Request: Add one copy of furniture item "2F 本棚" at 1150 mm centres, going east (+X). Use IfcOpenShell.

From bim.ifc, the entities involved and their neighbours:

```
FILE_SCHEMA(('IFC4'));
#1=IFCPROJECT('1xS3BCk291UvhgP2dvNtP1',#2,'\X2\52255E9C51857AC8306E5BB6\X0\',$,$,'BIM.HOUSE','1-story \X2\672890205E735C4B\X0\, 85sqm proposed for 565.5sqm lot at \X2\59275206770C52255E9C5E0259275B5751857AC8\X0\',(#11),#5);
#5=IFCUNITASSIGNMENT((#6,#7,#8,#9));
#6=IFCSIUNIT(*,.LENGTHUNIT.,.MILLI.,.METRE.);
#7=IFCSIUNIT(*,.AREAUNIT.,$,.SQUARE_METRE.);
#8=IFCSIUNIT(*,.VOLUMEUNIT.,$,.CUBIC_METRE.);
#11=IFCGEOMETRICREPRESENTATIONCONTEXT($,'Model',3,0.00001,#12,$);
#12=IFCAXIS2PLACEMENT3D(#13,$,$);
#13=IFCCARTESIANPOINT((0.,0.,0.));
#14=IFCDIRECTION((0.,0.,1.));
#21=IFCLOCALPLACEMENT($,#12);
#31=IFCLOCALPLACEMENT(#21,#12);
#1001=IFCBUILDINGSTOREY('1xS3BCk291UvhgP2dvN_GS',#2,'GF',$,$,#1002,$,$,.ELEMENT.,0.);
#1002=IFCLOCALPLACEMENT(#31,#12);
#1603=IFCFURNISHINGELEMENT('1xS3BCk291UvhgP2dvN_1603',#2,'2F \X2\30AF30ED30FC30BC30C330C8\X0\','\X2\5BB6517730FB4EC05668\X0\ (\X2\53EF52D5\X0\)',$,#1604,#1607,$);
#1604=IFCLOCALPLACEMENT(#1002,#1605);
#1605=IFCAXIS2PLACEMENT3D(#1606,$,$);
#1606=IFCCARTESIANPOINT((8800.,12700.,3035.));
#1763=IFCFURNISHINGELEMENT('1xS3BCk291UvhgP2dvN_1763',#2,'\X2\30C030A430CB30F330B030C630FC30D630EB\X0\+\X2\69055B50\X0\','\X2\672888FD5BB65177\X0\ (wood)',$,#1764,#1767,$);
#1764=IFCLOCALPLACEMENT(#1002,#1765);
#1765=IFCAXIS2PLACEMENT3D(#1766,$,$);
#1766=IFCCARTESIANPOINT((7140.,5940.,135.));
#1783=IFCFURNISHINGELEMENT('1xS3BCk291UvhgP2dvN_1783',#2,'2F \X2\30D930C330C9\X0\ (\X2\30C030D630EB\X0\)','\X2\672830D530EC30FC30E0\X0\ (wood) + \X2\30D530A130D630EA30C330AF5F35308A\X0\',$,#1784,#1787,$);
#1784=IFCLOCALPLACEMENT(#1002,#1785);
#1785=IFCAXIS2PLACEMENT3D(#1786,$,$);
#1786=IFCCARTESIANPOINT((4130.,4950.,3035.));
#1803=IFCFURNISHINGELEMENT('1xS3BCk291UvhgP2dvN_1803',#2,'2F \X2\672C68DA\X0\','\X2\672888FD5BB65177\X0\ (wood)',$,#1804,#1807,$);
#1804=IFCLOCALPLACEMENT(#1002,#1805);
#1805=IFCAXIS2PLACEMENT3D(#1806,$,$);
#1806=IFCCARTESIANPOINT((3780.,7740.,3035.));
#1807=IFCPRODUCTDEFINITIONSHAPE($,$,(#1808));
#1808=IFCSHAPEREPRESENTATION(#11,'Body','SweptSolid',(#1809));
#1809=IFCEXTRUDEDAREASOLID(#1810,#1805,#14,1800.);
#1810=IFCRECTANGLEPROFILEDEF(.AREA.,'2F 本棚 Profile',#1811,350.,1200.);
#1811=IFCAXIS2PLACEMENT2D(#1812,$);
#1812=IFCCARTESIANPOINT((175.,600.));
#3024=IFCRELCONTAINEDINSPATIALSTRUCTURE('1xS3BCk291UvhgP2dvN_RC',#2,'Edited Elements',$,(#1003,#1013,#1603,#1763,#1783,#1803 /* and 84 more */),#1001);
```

```python
import numpy as np
import ifcopenshell
import ifcopenshell.api.geometry
import ifcopenshell.api.root
import ifcopenshell.util.element
import ifcopenshell.util.placement

model = ifcopenshell.open("bim.ifc")


def reuse_history(source, copy):
    """copy_class also copies each property set's owner history, people and application; keep the originals."""
    for rel in copy.IsDefinedBy:
        if rel.is_a("IfcRelDefinesByProperties") and (history := rel.RelatingPropertyDefinition.OwnerHistory):
            rel.RelatingPropertyDefinition.OwnerHistory = source.OwnerHistory
            ifcopenshell.util.element.remove_deep2(model, history)


source = model.by_id(1803)
base = ifcopenshell.util.placement.get_local_placement(source.ObjectPlacement)
step = np.array([1.0, 0.0, 0.0]) * 1150.0

for i in range(1, 2):
    copy = ifcopenshell.api.root.copy_class(model, product=source)
    copy.Representation = ifcopenshell.util.element.copy_deep(
        model, source.Representation, exclude=["IfcGeometricRepresentationContext", "IfcRepresentationMap"]
    )
    reuse_history(source, copy)
    matrix = base.copy()
    matrix[:3, 3] += i * step
    print("added at", matrix[:3, 3].round(3) + 0.0)
    ifcopenshell.api.geometry.edit_object_placement(model, product=copy, matrix=matrix, is_si=False)

model.write("bim_v2.ifc")
```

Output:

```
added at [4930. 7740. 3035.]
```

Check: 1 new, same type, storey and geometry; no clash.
